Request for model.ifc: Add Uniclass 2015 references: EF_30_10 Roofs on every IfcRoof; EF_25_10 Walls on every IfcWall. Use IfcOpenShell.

First a look at what the model holds.

```python
import ifcopenshell

model = ifcopenshell.open("model.ifc")
print(model.schema)
print("classifications:", [c.Name for c in model.by_type("IfcClassification")])
for ifc_class in ("IfcDoor", "IfcRoof", "IfcStair", "IfcWall", "IfcWindow"):
    print(ifc_class, len(model.by_type(ifc_class)))
```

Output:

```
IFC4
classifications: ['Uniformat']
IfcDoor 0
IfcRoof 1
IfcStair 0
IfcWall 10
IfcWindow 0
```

```python
import ifcopenshell
import ifcopenshell.api.classification

model = ifcopenshell.open("model.ifc")

system = ifcopenshell.api.classification.add_classification(model, classification="Uniclass 2015")

codes = {
    "IfcRoof": ("EF_30_10", "Roofs"),
    "IfcWall": ("EF_25_10", "Walls"),
}
for ifc_class, (code, name) in codes.items():
    products = model.by_type(ifc_class)
    ifcopenshell.api.classification.add_reference(
        model, products=products, classification=system, identification=code, name=name
    )
    print(code, len(products))

model.write("model_v2.ifc")
```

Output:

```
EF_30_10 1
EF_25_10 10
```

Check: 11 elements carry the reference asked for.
